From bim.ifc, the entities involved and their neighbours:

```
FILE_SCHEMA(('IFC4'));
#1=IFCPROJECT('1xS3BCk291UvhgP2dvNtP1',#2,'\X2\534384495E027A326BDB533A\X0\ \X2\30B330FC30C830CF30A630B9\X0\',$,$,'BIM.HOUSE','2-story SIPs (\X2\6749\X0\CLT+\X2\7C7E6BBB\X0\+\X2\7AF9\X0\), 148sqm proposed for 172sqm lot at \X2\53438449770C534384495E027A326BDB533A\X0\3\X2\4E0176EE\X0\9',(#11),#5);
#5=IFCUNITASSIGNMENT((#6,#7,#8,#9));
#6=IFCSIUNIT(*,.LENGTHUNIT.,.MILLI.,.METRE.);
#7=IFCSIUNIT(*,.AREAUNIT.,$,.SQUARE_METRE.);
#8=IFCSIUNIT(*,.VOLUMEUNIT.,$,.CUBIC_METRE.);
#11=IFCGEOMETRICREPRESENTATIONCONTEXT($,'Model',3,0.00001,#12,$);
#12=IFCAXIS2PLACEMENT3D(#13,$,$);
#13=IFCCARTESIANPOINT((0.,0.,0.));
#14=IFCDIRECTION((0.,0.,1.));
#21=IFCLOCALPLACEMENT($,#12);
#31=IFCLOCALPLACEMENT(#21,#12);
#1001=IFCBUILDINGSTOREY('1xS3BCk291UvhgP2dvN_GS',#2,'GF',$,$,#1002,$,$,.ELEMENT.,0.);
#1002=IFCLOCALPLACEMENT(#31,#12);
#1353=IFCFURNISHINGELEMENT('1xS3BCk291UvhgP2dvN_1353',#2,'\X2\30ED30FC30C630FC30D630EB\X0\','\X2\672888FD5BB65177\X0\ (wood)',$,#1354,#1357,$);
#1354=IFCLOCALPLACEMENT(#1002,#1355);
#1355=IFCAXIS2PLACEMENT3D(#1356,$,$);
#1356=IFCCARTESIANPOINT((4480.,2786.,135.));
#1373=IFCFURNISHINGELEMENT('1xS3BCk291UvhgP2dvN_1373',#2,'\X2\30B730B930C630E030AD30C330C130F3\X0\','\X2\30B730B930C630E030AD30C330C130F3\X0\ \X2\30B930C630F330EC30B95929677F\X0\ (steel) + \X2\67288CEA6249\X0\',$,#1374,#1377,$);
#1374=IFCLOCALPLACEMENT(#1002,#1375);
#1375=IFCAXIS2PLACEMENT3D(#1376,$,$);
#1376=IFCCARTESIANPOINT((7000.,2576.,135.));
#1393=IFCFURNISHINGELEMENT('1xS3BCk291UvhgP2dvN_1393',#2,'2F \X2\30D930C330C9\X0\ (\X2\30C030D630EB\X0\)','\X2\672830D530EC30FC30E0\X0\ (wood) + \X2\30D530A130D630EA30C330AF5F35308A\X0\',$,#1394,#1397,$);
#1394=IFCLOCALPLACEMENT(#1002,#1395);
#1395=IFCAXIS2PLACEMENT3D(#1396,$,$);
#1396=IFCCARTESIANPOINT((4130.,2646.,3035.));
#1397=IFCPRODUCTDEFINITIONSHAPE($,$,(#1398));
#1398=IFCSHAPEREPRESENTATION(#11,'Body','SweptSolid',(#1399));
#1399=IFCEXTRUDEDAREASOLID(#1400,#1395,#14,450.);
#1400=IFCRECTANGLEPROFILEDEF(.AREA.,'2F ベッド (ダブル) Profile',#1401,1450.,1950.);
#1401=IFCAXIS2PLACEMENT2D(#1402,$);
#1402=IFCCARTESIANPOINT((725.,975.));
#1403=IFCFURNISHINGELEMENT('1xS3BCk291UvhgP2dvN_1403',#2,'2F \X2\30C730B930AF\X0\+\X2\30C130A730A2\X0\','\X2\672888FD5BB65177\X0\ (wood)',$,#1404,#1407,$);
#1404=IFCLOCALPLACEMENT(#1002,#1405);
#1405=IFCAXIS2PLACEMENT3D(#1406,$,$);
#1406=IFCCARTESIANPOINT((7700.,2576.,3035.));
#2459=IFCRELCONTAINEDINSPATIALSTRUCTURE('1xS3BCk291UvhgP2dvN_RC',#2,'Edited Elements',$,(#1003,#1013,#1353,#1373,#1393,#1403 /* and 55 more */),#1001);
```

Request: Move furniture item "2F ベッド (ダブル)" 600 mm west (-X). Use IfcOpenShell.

```python
import ifcopenshell
import ifcopenshell.api.geometry
import ifcopenshell.util.placement
import ifcopenshell.util.unit

model = ifcopenshell.open("bim.ifc")
unit_scale = ifcopenshell.util.unit.calculate_unit_scale(model)

item = model.by_guid("1xS3BCk291UvhgP2dvN_1393")
matrix = ifcopenshell.util.placement.get_local_placement(item.ObjectPlacement)
matrix[0, 3] -= 0.6 / unit_scale
ifcopenshell.api.geometry.edit_object_placement(model, product=item, matrix=matrix, is_si=False)

print(ifcopenshell.util.placement.get_local_placement(item.ObjectPlacement).round(3) + 0.0)

model.write("bim_edited.ifc")
```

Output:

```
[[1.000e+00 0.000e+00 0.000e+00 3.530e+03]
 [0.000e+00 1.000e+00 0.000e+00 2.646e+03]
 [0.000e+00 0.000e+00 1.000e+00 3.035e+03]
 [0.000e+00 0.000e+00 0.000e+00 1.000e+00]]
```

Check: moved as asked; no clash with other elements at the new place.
